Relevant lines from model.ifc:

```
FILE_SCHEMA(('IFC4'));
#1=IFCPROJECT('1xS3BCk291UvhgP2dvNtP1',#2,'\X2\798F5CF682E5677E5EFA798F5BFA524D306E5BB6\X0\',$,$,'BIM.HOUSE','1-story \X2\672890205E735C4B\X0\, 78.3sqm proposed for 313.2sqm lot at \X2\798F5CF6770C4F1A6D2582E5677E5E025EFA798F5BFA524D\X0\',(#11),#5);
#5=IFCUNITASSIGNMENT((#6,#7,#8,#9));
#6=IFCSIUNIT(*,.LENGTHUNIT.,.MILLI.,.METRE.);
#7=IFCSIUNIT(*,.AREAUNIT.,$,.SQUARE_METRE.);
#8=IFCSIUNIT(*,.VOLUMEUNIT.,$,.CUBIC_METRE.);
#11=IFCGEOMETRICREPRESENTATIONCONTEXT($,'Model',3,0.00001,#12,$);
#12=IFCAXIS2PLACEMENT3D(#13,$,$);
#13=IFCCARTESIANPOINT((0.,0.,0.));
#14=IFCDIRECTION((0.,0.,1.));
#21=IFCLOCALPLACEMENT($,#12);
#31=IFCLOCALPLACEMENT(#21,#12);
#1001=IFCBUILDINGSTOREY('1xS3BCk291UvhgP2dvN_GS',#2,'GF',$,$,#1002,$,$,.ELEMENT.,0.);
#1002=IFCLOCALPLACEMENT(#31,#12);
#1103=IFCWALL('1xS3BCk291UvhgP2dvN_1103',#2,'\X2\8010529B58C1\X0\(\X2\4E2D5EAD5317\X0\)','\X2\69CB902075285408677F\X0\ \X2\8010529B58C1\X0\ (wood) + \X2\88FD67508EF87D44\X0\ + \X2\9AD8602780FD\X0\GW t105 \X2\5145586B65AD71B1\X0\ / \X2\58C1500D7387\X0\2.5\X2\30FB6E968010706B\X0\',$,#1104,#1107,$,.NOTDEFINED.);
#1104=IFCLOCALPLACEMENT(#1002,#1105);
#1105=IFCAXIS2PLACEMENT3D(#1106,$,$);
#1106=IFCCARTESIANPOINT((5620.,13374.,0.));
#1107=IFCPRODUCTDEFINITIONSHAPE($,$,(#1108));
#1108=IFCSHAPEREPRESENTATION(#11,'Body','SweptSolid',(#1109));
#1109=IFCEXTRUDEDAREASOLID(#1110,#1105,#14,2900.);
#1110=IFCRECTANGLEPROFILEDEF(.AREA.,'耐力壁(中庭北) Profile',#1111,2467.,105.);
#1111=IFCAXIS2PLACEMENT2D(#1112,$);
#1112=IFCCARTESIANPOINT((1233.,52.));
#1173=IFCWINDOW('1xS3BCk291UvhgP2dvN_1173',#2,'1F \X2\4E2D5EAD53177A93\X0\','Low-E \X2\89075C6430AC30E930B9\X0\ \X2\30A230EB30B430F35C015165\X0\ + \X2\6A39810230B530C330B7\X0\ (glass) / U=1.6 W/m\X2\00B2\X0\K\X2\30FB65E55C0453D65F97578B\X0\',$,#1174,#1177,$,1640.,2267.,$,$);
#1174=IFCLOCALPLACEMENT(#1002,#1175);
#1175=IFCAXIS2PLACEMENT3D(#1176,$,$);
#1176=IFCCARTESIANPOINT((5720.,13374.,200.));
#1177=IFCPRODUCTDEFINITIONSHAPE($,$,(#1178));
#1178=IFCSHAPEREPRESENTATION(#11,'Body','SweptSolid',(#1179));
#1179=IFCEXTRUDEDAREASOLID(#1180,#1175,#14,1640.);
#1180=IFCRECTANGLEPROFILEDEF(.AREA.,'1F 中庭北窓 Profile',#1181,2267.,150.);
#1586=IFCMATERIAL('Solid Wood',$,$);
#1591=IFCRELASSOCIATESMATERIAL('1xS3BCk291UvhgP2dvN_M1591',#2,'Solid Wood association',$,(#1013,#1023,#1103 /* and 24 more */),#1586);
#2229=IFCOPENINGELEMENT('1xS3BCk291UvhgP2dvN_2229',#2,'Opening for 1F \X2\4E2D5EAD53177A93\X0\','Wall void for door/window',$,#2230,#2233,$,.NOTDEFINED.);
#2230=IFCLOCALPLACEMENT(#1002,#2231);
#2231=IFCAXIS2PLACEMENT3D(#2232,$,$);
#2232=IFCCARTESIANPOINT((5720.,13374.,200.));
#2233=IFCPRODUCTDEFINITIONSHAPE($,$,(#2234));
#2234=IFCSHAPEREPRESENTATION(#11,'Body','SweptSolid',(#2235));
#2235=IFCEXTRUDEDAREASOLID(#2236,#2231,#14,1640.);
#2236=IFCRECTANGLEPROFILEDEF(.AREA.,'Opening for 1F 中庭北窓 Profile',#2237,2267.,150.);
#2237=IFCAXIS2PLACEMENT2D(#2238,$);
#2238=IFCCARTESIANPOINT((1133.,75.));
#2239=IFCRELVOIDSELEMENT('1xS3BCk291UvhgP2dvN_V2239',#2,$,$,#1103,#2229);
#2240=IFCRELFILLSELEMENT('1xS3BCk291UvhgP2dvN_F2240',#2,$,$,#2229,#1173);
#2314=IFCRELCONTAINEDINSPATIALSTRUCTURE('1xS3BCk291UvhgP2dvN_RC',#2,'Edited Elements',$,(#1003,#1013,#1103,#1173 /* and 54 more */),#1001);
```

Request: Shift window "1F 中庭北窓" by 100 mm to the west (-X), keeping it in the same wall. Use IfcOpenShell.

```python
import ifcopenshell
import ifcopenshell.api.geometry
import ifcopenshell.util.placement
import ifcopenshell.util.unit

model = ifcopenshell.open("model.ifc")
unit_scale = ifcopenshell.util.unit.calculate_unit_scale(model)

window = model.by_guid("1xS3BCk291UvhgP2dvN_1173")
opening = window.FillsVoids[0].RelatingOpeningElement
wall = opening.VoidsElements[0].RelatingBuildingElement

wall_matrix = ifcopenshell.util.placement.get_local_placement(wall.ObjectPlacement)
shift = wall_matrix[:3, 0] * -0.1 / unit_scale
before = ifcopenshell.util.placement.get_local_placement(window.ObjectPlacement)[:3, 3].copy()

# The window is not placed relative to its opening, so move both.
for product in (opening, window):
    matrix = ifcopenshell.util.placement.get_local_placement(product.ObjectPlacement)
    matrix[:3, 3] += shift
    ifcopenshell.api.geometry.edit_object_placement(model, product=product, matrix=matrix, is_si=False)

after = ifcopenshell.util.placement.get_local_placement(window.ObjectPlacement)[:3, 3]
print("window moved by", (after - before).round(3) + 0.0)

model.write("model_v2.ifc")
```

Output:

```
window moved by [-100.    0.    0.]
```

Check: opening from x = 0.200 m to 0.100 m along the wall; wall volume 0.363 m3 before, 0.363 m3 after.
